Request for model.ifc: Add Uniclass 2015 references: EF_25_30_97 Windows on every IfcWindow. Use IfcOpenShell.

First a look at what the model holds.

```python
import ifcopenshell

model = ifcopenshell.open("model.ifc")
print(model.schema)
print("classifications:", [c.Name for c in model.by_type("IfcClassification")])
for ifc_class in ("IfcDoor", "IfcRoof", "IfcStair", "IfcWall", "IfcWindow"):
    print(ifc_class, len(model.by_type(ifc_class)))
```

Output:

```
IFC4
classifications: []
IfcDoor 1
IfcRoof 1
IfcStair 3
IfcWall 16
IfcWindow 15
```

```python
import ifcopenshell
import ifcopenshell.api.classification

model = ifcopenshell.open("model.ifc")

system = ifcopenshell.api.classification.add_classification(model, classification="Uniclass 2015")

codes = {
    "IfcWindow": ("EF_25_30_97", "Windows"),
}
for ifc_class, (code, name) in codes.items():
    products = model.by_type(ifc_class)
    ifcopenshell.api.classification.add_reference(
        model, products=products, classification=system, identification=code, name=name
    )
    print(code, len(products))

model.write("model_edited.ifc")
```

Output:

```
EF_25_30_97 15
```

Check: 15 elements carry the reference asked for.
